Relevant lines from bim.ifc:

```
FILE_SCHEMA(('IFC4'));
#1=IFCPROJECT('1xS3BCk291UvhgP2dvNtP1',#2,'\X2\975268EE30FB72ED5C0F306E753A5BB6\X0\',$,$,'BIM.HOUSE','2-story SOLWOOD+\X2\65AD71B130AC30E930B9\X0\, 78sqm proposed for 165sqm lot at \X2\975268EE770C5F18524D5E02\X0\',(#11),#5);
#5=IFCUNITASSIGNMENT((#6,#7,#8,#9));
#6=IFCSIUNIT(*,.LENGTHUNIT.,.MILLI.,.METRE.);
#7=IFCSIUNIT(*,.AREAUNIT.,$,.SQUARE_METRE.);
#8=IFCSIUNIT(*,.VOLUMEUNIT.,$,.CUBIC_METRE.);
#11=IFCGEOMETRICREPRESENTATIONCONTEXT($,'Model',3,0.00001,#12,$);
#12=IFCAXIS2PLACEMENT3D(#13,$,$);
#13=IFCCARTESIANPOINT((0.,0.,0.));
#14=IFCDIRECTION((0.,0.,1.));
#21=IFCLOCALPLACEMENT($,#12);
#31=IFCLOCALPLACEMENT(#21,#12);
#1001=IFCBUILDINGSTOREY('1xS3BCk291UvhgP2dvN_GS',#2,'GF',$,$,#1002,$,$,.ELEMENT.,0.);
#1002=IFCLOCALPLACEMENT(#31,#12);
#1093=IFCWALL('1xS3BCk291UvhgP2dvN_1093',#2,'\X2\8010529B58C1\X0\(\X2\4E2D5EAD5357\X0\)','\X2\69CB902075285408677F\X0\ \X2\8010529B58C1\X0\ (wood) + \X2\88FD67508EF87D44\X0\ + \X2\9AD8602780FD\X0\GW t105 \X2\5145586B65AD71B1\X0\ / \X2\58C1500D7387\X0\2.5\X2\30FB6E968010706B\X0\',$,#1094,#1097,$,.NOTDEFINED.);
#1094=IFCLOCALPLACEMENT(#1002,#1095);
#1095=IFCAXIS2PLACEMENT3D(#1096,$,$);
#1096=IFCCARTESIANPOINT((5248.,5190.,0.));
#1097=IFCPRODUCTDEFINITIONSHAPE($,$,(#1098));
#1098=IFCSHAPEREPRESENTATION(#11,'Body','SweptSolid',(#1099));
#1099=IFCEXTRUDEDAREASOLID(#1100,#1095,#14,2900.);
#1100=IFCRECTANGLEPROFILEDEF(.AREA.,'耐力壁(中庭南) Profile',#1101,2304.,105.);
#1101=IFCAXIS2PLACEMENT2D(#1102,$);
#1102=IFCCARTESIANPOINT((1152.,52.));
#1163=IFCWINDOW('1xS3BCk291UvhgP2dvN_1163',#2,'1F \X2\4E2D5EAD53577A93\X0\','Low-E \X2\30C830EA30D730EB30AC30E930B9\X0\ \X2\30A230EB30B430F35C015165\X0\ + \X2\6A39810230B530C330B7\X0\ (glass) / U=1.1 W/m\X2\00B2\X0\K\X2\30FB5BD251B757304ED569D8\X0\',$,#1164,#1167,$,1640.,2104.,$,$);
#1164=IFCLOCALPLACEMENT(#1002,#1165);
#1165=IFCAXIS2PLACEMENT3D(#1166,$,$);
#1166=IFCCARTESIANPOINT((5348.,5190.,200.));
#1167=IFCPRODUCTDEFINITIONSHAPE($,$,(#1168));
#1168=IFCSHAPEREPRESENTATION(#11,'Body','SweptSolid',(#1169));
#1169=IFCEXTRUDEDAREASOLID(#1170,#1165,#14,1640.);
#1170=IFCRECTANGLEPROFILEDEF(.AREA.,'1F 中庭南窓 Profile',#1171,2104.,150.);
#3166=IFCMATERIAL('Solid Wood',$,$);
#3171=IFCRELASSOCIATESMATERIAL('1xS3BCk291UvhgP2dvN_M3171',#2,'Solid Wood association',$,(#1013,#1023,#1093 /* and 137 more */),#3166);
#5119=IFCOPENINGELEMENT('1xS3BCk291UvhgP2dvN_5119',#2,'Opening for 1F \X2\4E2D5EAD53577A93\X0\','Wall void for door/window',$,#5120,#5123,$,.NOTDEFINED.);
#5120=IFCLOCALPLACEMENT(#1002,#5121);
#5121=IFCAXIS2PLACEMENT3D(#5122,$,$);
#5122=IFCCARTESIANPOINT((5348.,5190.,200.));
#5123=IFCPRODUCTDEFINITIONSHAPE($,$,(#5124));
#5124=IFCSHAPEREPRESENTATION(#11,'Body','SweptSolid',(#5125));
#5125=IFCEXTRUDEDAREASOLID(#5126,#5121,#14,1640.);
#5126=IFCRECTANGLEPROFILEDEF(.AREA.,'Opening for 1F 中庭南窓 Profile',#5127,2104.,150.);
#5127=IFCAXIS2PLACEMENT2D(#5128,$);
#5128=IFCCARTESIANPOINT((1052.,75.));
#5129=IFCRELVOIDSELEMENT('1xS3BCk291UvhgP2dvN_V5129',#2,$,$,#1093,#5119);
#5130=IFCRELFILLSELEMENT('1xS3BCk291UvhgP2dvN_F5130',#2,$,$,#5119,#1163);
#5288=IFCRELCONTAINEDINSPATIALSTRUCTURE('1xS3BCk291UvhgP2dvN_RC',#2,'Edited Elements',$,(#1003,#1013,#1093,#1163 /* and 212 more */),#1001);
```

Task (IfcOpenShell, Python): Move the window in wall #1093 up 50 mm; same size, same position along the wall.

```python
import numpy as np
import ifcopenshell
import ifcopenshell.api.geometry
import ifcopenshell.util.placement
import ifcopenshell.util.unit

model = ifcopenshell.open("bim.ifc")
unit_scale = ifcopenshell.util.unit.calculate_unit_scale(model)

window = model.by_guid("1xS3BCk291UvhgP2dvN_1163")
opening = window.FillsVoids[0].RelatingOpeningElement
dz = 50.0

shift = np.array([0.0, 0.0, dz])
# The window is not placed relative to its opening, so move both.
for product in (opening, window):
    matrix = ifcopenshell.util.placement.get_local_placement(product.ObjectPlacement)
    matrix[:3, 3] += shift
    ifcopenshell.api.geometry.edit_object_placement(model, product=product, matrix=matrix, is_si=False)

print(f"moved by {dz * unit_scale:+.3f} m")

model.write("bim_v2.ifc")
```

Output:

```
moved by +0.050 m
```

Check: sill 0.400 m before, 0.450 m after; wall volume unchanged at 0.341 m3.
